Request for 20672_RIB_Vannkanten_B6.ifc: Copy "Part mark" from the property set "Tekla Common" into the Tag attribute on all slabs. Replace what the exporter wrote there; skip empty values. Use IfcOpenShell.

First a look at what the model holds.

```python
import ifcopenshell
import ifcopenshell.util.element

model = ifcopenshell.open("20672_RIB_Vannkanten_B6.ifc")
print(model.schema)
slabs = model.by_type("IfcSlab")
print(len(slabs), "slabs")
for e in slabs[:8]:
    source = ifcopenshell.util.element.get_pset(e, "Tekla Common", "Part mark")
    target = e.Tag
    print(e.id(), repr(source), repr(target), sep=" | ")
```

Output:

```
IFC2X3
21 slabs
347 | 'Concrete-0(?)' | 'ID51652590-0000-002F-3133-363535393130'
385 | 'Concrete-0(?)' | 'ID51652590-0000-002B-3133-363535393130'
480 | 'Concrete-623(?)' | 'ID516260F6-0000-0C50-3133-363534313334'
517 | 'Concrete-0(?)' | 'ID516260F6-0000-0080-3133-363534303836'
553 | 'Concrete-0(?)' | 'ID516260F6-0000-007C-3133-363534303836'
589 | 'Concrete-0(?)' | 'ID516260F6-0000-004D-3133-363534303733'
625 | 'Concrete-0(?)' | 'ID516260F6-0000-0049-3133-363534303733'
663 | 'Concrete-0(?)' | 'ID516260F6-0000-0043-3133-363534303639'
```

```python
import ifcopenshell
import ifcopenshell.util.element

model = ifcopenshell.open("20672_RIB_Vannkanten_B6.ifc")

count = 0
for e in model.by_type("IfcSlab"):
    value = ifcopenshell.util.element.get_pset(e, "Tekla Common", "Part mark")
    current = e.Tag
    if not value or not value.strip() or current == value:
        continue
    e.Tag = value
    count += 1

print(count, "slabs updated")

model.write("20672_RIB_Vannkanten_B6-out.ifc")
```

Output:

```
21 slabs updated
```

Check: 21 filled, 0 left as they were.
